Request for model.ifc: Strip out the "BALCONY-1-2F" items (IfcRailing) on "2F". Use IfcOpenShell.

First a look at what the model holds.

```python
import ifcopenshell
import ifcopenshell.util.element

model = ifcopenshell.open("model.ifc")
print(model.schema)
storey = next(s for s in model.by_type("IfcBuildingStorey") if s.Name == "2F")
railings = [e for e in ifcopenshell.util.element.get_decomposition(storey) if e.is_a("IfcRailing")]
seen = {}
for e in railings:
    element_type = ifcopenshell.util.element.get_type(e)
    name = element_type.Name if element_type not in (None, e) else None
    seen[name] = seen.get(name, 0) + 1
for name, count in sorted(seen.items(), key=str):
    print(count, "x", name)
```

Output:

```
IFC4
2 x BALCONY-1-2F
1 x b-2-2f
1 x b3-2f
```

```python
import ifcopenshell
import ifcopenshell.api.root
import ifcopenshell.util.element

model = ifcopenshell.open("model.ifc")

storey = next(s for s in model.by_type("IfcBuildingStorey") if s.Name == "2F")
railings = [e for e in ifcopenshell.util.element.get_decomposition(storey) if e.is_a("IfcRailing")]
targets = [e for e in railings if (t := ifcopenshell.util.element.get_type(e)) not in (None, e) and t.Name == "BALCONY-1-2F"]

for e in targets:
    ifcopenshell.api.root.remove_product(model, product=e)
print(len(targets), "removed")

model.write("model_updated.ifc")
```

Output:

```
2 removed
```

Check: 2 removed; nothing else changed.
